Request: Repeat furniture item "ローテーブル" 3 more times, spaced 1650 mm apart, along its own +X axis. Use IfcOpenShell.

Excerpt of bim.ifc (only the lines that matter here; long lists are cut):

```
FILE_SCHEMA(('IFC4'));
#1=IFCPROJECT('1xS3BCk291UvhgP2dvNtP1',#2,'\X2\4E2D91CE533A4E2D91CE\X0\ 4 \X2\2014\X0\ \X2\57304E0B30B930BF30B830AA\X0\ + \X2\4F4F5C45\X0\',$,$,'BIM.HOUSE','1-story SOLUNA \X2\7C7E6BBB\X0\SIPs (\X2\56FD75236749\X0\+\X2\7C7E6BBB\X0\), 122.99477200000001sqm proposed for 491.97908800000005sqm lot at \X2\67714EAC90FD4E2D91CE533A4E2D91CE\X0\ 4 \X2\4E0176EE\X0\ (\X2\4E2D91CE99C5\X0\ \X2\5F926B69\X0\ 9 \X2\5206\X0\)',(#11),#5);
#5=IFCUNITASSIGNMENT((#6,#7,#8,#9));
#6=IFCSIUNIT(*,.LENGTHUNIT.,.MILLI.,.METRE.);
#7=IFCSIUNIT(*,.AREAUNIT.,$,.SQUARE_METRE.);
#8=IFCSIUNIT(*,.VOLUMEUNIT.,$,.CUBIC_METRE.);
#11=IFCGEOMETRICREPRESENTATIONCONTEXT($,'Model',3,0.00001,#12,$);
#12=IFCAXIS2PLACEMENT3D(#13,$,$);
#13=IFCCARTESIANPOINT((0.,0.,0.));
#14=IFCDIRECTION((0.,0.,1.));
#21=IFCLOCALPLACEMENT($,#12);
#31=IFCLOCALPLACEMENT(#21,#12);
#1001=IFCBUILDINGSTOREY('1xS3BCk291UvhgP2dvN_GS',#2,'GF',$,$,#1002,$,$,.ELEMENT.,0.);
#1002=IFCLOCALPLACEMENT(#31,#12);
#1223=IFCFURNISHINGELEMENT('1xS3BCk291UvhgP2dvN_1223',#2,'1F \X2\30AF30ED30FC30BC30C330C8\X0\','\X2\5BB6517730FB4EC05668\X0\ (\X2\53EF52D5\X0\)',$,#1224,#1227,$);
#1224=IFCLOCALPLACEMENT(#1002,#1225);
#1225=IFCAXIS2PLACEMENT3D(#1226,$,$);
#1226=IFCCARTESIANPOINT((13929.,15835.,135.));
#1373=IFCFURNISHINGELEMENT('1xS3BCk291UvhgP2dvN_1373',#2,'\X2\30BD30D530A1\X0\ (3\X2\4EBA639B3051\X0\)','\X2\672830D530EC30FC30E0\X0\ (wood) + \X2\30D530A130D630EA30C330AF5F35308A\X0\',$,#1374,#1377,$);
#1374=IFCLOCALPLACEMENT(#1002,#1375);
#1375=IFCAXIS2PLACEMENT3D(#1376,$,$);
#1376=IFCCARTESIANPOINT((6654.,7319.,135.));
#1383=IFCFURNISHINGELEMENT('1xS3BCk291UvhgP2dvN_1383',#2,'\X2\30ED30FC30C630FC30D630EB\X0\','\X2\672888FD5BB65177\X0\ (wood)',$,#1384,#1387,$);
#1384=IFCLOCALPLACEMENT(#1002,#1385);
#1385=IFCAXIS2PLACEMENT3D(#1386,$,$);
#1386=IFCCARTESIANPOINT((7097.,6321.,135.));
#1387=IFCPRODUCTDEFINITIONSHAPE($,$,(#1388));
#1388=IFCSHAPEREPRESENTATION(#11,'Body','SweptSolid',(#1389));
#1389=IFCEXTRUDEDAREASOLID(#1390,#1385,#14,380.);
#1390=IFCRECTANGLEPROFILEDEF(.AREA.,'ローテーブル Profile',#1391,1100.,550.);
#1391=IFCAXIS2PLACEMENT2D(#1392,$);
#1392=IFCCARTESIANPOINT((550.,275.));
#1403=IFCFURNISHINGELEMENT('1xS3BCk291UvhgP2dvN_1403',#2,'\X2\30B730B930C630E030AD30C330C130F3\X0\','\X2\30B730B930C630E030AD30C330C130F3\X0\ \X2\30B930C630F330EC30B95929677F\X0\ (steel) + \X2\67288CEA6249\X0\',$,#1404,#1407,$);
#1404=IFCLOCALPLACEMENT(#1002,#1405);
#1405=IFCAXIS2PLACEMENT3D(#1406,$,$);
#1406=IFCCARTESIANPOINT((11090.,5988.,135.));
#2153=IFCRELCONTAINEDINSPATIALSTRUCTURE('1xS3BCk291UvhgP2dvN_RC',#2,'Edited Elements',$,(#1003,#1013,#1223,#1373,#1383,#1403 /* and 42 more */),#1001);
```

```python
import ifcopenshell
import ifcopenshell.api.geometry
import ifcopenshell.api.root
import ifcopenshell.util.element
import ifcopenshell.util.placement

model = ifcopenshell.open("bim.ifc")


def reuse_history(source, copy):
    """copy_class also copies each property set's owner history, people and application; keep the originals."""
    for rel in copy.IsDefinedBy:
        if rel.is_a("IfcRelDefinesByProperties") and (history := rel.RelatingPropertyDefinition.OwnerHistory):
            rel.RelatingPropertyDefinition.OwnerHistory = source.OwnerHistory
            ifcopenshell.util.element.remove_deep2(model, history)


source = model.by_id(1383)
base = ifcopenshell.util.placement.get_local_placement(source.ObjectPlacement)
step = base[:3, 0] * 1650.0

for i in range(1, 4):
    copy = ifcopenshell.api.root.copy_class(model, product=source)
    copy.Representation = ifcopenshell.util.element.copy_deep(
        model, source.Representation, exclude=["IfcGeometricRepresentationContext", "IfcRepresentationMap"]
    )
    reuse_history(source, copy)
    matrix = base.copy()
    matrix[:3, 3] += i * step
    print("added at", matrix[:3, 3].round(3) + 0.0)
    ifcopenshell.api.geometry.edit_object_placement(model, product=copy, matrix=matrix, is_si=False)

model.write("bim_edited.ifc")
```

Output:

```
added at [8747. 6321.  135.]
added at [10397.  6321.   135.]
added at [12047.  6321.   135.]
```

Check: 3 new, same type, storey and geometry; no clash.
